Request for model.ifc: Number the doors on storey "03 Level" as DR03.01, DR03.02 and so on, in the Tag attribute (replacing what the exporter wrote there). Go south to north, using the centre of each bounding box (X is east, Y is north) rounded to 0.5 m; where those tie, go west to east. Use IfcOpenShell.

First a look at what the model holds.

```python
import ifcopenshell
import ifcopenshell.util.element
import ifcopenshell.util.placement

model = ifcopenshell.open("model.ifc")
print(model.schema)
storey = next(s for s in model.by_type("IfcBuildingStorey") if s.Name == "03 Level")
doors = [e for e in ifcopenshell.util.element.get_decomposition(storey) if e.is_a("IfcDoor")]
for e in sorted(doors, key=lambda e: e.id()):
    origin = ifcopenshell.util.placement.get_local_placement(e.ObjectPlacement)[:3, 3]
    print(e.id(), e.Tag, e.Name, origin.round(2) + 0.0, sep=" | ")
```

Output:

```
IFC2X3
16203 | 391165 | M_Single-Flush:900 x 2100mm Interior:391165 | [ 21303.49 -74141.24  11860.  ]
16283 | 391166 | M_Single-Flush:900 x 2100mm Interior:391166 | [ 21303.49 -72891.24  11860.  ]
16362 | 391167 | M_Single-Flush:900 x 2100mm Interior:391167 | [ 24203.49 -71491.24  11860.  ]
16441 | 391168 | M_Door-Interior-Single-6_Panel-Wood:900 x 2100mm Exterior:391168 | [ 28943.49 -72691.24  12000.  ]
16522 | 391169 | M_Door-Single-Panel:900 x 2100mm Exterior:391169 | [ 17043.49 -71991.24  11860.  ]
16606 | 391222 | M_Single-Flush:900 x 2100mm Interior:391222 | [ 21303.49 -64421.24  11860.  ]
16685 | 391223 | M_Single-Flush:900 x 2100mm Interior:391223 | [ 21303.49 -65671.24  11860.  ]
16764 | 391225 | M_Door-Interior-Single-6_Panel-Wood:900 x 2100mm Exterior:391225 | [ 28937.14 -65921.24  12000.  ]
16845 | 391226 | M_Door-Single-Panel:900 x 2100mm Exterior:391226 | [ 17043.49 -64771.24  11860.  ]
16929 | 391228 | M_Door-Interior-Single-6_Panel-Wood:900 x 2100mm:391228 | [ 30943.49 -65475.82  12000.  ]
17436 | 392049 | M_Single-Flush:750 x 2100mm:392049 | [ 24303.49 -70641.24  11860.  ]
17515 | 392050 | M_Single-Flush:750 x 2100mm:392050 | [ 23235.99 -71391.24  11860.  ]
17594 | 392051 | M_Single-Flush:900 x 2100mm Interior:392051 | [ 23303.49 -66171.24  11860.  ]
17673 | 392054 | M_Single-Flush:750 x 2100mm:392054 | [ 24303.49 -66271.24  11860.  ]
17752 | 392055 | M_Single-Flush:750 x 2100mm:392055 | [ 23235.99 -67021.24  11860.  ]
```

```python
import ifcopenshell
import ifcopenshell.geom
import ifcopenshell.util.element
import ifcopenshell.util.shape

model = ifcopenshell.open("model.ifc")
settings = ifcopenshell.geom.settings()
settings.set("use-world-coords", True)


def centre(element):
    shape = ifcopenshell.geom.create_shape(settings, element)
    return ifcopenshell.util.shape.get_bbox_centroid(shape.geometry)


storey = next(s for s in model.by_type("IfcBuildingStorey") if s.Name == "03 Level")
doors = [e for e in ifcopenshell.util.element.get_decomposition(storey) if e.is_a("IfcDoor")]

# Insertion points can sit at a corner or the storey origin, so sort by the geometry (in metres).
centres = {e: centre(e) for e in doors}
doors.sort(key=lambda e: (round(centres[e][1] / 0.5), centres[e][0]))

for i, e in enumerate(doors, start=1):
    number = f"DR03.{i:02d}"
    e.Tag = number
    print(e.id(), number)

model.write("model_edited.ifc")
```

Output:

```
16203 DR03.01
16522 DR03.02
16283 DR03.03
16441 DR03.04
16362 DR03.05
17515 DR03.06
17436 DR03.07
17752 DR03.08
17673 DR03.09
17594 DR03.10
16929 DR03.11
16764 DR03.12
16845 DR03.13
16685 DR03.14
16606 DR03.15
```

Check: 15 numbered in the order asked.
